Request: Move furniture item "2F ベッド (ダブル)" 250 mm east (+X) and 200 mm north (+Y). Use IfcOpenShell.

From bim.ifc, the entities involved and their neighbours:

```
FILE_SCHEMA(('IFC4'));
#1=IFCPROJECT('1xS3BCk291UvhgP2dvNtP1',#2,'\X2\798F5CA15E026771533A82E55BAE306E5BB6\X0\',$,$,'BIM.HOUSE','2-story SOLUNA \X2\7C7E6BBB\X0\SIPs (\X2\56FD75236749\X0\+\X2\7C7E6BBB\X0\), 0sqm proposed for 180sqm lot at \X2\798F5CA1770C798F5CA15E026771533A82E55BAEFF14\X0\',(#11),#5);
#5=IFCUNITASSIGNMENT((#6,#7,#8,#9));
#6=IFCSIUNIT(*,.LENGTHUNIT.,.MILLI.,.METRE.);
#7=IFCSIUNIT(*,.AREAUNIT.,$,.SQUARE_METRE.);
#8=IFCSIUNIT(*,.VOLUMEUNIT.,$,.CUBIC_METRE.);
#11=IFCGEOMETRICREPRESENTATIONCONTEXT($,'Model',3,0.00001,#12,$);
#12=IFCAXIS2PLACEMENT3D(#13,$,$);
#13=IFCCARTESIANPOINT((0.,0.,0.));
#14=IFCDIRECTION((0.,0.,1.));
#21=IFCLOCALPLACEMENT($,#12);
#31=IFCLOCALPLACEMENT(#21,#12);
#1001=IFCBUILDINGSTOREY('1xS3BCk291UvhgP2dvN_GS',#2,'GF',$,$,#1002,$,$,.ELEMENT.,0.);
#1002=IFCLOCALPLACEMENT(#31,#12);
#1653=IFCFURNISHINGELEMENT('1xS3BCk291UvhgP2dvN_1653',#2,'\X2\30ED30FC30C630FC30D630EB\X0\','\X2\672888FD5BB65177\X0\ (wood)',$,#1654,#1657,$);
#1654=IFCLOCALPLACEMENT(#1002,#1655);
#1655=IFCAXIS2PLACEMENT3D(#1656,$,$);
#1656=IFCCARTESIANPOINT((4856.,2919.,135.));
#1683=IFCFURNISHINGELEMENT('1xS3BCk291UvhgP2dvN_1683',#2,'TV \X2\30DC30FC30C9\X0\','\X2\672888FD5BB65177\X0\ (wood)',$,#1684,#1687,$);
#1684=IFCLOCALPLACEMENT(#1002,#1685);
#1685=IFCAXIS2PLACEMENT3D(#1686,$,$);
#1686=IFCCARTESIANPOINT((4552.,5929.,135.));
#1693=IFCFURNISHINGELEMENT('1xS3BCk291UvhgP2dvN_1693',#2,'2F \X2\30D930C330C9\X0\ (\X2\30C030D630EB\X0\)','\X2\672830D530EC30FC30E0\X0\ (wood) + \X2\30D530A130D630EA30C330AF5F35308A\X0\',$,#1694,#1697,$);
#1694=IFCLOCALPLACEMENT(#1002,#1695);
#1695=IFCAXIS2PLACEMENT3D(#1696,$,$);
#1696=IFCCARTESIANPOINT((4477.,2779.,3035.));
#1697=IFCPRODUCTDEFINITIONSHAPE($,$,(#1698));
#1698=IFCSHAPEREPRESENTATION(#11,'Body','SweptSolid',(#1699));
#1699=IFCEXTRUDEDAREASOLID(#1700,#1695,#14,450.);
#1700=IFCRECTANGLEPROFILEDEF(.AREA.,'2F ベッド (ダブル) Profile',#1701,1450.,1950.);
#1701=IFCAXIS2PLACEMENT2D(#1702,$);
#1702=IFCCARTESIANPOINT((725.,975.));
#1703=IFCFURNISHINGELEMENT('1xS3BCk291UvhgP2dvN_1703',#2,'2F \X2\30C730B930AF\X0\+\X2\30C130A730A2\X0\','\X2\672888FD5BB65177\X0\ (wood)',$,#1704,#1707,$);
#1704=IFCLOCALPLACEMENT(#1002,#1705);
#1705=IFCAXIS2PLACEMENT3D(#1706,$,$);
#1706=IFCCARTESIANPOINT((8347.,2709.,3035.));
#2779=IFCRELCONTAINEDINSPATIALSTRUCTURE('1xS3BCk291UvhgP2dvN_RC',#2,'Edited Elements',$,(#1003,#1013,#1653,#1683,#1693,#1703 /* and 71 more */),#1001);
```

```python
import ifcopenshell
import ifcopenshell.api.geometry
import ifcopenshell.util.placement
import ifcopenshell.util.unit

model = ifcopenshell.open("bim.ifc")
unit_scale = ifcopenshell.util.unit.calculate_unit_scale(model)

item = model.by_guid("1xS3BCk291UvhgP2dvN_1693")
matrix = ifcopenshell.util.placement.get_local_placement(item.ObjectPlacement)
matrix[0, 3] += 0.25 / unit_scale
matrix[1, 3] += 0.2 / unit_scale
ifcopenshell.api.geometry.edit_object_placement(model, product=item, matrix=matrix, is_si=False)

print(ifcopenshell.util.placement.get_local_placement(item.ObjectPlacement).round(3) + 0.0)

model.write("bim_updated.ifc")
```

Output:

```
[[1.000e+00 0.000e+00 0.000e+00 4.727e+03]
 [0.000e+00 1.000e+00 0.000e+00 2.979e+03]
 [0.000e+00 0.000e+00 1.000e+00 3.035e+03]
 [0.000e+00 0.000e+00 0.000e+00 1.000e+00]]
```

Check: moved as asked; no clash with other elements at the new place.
